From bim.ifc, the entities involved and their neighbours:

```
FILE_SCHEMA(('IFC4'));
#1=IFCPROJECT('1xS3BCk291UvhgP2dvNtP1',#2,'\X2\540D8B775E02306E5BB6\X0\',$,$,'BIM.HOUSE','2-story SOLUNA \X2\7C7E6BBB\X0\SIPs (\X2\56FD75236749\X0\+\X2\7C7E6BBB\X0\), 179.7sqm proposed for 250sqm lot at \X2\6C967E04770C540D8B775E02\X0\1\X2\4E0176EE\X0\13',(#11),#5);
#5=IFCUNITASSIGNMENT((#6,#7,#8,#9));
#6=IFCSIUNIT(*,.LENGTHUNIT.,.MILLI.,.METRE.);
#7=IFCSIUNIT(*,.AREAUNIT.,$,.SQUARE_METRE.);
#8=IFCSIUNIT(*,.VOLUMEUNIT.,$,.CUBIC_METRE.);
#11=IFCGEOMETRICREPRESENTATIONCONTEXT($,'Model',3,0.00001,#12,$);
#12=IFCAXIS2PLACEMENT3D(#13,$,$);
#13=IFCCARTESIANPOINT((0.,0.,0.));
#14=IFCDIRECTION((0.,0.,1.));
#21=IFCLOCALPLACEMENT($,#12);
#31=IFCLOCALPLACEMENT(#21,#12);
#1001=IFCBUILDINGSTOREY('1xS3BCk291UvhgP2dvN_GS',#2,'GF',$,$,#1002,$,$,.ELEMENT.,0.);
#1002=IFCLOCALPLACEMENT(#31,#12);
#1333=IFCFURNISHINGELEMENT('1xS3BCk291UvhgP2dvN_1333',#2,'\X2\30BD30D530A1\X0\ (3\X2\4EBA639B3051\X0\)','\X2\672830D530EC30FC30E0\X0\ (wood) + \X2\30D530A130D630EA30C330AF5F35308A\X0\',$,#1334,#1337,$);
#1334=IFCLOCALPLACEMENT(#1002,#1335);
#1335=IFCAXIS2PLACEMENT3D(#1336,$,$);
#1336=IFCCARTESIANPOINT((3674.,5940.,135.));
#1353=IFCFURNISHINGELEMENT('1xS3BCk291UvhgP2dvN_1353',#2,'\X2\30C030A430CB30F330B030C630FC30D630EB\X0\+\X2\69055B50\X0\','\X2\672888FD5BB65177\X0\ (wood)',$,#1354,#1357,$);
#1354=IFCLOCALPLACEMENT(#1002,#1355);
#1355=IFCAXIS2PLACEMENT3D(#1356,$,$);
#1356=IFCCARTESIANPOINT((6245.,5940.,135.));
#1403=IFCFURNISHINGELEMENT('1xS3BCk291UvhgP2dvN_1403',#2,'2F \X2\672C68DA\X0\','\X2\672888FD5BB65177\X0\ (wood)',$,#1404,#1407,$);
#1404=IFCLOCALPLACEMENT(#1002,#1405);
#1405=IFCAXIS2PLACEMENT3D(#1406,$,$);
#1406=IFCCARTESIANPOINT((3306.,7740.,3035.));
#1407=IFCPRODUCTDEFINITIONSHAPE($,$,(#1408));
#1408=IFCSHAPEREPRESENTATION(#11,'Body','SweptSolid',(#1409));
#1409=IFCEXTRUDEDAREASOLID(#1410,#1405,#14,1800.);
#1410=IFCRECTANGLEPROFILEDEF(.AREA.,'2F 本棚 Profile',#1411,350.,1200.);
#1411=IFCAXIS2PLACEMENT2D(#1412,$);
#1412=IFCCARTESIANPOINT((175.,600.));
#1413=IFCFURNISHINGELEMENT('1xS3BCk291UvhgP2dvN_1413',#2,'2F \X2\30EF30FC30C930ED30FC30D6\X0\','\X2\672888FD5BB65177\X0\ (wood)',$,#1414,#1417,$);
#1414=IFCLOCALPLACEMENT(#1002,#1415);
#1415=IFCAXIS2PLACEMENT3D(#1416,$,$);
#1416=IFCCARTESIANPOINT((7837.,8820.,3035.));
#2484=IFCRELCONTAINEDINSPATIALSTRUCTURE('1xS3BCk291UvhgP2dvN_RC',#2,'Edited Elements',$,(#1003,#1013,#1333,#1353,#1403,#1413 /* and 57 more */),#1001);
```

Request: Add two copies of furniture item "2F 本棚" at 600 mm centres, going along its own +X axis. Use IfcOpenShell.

```python
import ifcopenshell
import ifcopenshell.api.geometry
import ifcopenshell.api.root
import ifcopenshell.util.element
import ifcopenshell.util.placement

model = ifcopenshell.open("bim.ifc")


def reuse_history(source, copy):
    """copy_class also copies each property set's owner history, people and application; keep the originals."""
    for rel in copy.IsDefinedBy:
        if rel.is_a("IfcRelDefinesByProperties") and (history := rel.RelatingPropertyDefinition.OwnerHistory):
            rel.RelatingPropertyDefinition.OwnerHistory = source.OwnerHistory
            ifcopenshell.util.element.remove_deep2(model, history)


source = model.by_guid("1xS3BCk291UvhgP2dvN_1403")
base = ifcopenshell.util.placement.get_local_placement(source.ObjectPlacement)
step = base[:3, 0] * 600.0

for i in range(1, 3):
    copy = ifcopenshell.api.root.copy_class(model, product=source)
    copy.Representation = ifcopenshell.util.element.copy_deep(
        model, source.Representation, exclude=["IfcGeometricRepresentationContext", "IfcRepresentationMap"]
    )
    reuse_history(source, copy)
    matrix = base.copy()
    matrix[:3, 3] += i * step
    print("added at", matrix[:3, 3].round(3) + 0.0)
    ifcopenshell.api.geometry.edit_object_placement(model, product=copy, matrix=matrix, is_si=False)

model.write("bim_updated.ifc")
```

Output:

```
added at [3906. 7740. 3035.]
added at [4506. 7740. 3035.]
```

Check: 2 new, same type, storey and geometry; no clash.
